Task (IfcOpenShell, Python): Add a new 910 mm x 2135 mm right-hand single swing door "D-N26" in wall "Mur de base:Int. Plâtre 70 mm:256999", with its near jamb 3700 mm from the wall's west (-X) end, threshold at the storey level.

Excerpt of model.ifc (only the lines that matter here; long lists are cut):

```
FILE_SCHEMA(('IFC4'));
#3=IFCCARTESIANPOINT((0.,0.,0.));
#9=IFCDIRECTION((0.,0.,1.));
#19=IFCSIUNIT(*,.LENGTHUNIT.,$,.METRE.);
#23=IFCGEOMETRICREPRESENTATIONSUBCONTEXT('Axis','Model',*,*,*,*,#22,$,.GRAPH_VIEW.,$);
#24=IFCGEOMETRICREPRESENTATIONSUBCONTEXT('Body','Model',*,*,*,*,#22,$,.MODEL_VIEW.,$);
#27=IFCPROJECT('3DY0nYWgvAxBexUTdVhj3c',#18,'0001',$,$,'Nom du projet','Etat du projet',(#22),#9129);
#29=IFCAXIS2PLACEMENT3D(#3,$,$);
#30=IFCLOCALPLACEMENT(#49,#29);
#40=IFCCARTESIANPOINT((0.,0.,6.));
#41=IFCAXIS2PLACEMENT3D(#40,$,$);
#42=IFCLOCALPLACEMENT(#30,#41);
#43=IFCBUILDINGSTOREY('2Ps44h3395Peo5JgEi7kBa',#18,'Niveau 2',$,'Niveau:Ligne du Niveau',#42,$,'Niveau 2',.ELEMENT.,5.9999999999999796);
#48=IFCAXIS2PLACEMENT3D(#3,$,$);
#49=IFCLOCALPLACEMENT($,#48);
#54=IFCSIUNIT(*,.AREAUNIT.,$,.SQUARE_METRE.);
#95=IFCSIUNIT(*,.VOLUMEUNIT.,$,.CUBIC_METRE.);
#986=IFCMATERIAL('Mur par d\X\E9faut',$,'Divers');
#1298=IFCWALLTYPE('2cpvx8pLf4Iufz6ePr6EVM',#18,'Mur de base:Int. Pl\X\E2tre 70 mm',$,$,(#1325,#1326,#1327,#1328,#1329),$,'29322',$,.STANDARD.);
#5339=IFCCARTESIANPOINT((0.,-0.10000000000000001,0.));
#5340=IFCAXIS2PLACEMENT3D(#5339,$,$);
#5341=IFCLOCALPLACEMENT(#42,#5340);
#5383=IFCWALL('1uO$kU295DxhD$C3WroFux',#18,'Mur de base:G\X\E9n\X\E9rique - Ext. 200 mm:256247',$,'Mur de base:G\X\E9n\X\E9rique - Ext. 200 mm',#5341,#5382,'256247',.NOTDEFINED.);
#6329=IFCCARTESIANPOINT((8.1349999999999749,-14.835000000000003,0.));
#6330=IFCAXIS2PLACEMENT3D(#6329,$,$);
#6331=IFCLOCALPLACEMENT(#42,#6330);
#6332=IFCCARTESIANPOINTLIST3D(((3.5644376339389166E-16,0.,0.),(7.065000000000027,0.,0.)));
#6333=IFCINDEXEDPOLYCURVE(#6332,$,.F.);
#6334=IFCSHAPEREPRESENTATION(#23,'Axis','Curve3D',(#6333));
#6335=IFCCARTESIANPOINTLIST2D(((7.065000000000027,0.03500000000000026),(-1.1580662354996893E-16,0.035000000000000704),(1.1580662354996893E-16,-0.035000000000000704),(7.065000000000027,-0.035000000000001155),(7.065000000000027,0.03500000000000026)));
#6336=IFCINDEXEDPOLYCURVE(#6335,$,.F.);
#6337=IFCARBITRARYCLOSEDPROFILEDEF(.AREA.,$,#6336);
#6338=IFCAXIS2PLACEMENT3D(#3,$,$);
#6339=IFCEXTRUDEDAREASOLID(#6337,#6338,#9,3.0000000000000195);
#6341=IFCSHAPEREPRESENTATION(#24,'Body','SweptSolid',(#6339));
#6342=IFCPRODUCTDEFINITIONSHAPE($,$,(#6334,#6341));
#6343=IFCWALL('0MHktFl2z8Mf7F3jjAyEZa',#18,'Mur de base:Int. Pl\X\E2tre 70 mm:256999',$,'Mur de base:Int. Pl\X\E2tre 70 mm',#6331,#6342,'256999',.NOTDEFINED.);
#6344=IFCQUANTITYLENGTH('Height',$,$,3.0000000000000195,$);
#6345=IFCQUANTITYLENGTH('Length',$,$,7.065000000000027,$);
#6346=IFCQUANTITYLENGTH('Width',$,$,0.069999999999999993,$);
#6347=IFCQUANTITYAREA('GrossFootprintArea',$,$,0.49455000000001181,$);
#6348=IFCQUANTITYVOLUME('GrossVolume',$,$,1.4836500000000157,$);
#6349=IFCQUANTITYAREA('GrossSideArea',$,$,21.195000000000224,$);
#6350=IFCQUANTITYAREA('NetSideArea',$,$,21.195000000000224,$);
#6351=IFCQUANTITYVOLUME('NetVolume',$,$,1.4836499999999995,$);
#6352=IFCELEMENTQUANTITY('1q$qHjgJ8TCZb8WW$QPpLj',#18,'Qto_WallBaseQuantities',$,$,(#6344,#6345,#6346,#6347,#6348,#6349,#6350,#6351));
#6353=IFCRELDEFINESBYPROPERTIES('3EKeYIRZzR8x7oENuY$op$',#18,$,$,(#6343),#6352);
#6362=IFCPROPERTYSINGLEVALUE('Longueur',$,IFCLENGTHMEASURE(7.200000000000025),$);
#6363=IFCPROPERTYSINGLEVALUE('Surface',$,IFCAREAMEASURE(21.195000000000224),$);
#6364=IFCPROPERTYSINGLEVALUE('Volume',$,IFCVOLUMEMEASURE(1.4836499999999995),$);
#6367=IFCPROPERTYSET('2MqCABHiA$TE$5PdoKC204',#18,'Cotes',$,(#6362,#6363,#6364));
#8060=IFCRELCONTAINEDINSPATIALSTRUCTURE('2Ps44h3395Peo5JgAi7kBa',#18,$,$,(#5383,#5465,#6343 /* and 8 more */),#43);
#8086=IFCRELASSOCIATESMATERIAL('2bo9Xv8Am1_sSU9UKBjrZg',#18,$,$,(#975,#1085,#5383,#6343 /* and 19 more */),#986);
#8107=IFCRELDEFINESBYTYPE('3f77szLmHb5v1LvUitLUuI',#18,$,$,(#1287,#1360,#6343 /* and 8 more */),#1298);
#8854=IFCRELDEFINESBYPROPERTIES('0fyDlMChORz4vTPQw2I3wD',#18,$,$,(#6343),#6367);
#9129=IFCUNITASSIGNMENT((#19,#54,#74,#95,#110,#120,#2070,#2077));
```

```python
import numpy as np
import ifcopenshell
import ifcopenshell.api.feature
import ifcopenshell.api.geometry
import ifcopenshell.api.pset
import ifcopenshell.api.root
import ifcopenshell.api.spatial
import ifcopenshell.geom
import ifcopenshell.util.element
import ifcopenshell.util.placement
import ifcopenshell.util.representation
import ifcopenshell.util.shape
import ifcopenshell.util.unit

model = ifcopenshell.open("model.ifc")
unit_scale = ifcopenshell.util.unit.calculate_unit_scale(model)
area_scale = ifcopenshell.util.unit.calculate_unit_scale(model, "AREAUNIT")
volume_scale = ifcopenshell.util.unit.calculate_unit_scale(model, "VOLUMEUNIT")
settings = ifcopenshell.geom.settings()


def volume(element):
    """Net volume in cubic metres, openings subtracted."""
    shape = ifcopenshell.geom.create_shape(settings, element)
    return ifcopenshell.util.shape.get_volume(shape.geometry)


wall = model.by_guid("0MHktFl2z8Mf7F3jjAyEZa")
storey = ifcopenshell.util.element.get_container(wall, ifc_class="IfcBuildingStorey")
context = ifcopenshell.util.representation.get_context(model, "Model", "Body", "MODEL_VIEW")
before = volume(wall)

width, height, from_end, sill = 0.91, 2.135, 3.7, 0.0  # metres

# The wall runs along its own X axis, and the end named is its -X end.
wall_shape = ifcopenshell.geom.create_shape(settings, wall)
x, y, z = ifcopenshell.util.shape.get_vertices(wall_shape.geometry).T
start = x.min() + from_end
face, thickness = float(y.min()), float(y.max() - y.min())
wall_matrix = ifcopenshell.util.placement.get_local_placement(wall.ObjectPlacement)
level = ifcopenshell.util.placement.get_local_placement(storey.ObjectPlacement)[2, 3]


def in_wall(x, y):
    """Placement at x, y metres in the wall's axes, at sill height."""
    matrix = wall_matrix.copy()
    matrix[:, 3] = wall_matrix @ np.array([x / unit_scale, y / unit_scale, 0.0, 1.0])
    matrix[2, 3] = level + sill / unit_scale
    return matrix


# Opening: a box that overshoots both wall faces by 50 mm.
opening = ifcopenshell.api.root.create_entity(model, ifc_class="IfcOpeningElement", predefined_type="OPENING")
box = ifcopenshell.api.geometry.add_wall_representation(
    model, context=context, length=width, height=height, thickness=thickness + 0.1
)
ifcopenshell.api.geometry.assign_representation(model, product=opening, representation=box)
ifcopenshell.api.geometry.edit_object_placement(model, product=opening, matrix=in_wall(start, face - 0.05), is_si=False)
ifcopenshell.api.feature.add_feature(model, feature=opening, element=wall)

door = ifcopenshell.api.root.create_entity(model, ifc_class="IfcDoor", name="D-N26", predefined_type="DOOR")
door.OverallWidth, door.OverallHeight = width / unit_scale, height / unit_scale
door.OperationType = "SINGLE_SWING_RIGHT"
body = ifcopenshell.api.geometry.add_door_representation(
    model,
    context=context,
    overall_width=door.OverallWidth,
    overall_height=door.OverallHeight,
    operation_type="SINGLE_SWING_RIGHT",
    lining_properties={"LiningDepth": thickness / unit_scale, "ThresholdDepth": thickness / unit_scale},
)
ifcopenshell.api.geometry.assign_representation(model, product=door, representation=body)
ifcopenshell.api.spatial.assign_container(model, products=[door], relating_structure=storey)
ifcopenshell.api.feature.add_filling(model, opening=opening, element=door)

# The lining spans the wall, so the door starts at the wall face.
ifcopenshell.api.geometry.edit_object_placement(model, product=door, matrix=in_wall(start, face), is_si=False)

after = volume(wall)

# Update the wall's stored quantities.
qto = model.by_id(ifcopenshell.util.element.get_pset(wall, "Qto_WallBaseQuantities", should_inherit=False)["id"])
ifcopenshell.api.pset.edit_qto(model, qto=qto, properties={
    "NetSideArea": after / thickness / area_scale,
    "NetVolume": after / volume_scale,
})
pset = model.by_id(ifcopenshell.util.element.get_pset(wall, "Cotes", should_inherit=False)["id"])
ifcopenshell.api.pset.edit_pset(model, pset=pset, properties={
    "Surface": model.create_entity("IfcAreaMeasure", after / thickness / area_scale),
    "Volume": model.create_entity("IfcVolumeMeasure", after / volume_scale),
})

print(f"wall volume {before:.3f} -> {after:.3f} m3")

model.write("model_edited.ifc")
```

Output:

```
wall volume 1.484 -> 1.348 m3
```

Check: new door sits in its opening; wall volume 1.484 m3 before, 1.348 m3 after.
